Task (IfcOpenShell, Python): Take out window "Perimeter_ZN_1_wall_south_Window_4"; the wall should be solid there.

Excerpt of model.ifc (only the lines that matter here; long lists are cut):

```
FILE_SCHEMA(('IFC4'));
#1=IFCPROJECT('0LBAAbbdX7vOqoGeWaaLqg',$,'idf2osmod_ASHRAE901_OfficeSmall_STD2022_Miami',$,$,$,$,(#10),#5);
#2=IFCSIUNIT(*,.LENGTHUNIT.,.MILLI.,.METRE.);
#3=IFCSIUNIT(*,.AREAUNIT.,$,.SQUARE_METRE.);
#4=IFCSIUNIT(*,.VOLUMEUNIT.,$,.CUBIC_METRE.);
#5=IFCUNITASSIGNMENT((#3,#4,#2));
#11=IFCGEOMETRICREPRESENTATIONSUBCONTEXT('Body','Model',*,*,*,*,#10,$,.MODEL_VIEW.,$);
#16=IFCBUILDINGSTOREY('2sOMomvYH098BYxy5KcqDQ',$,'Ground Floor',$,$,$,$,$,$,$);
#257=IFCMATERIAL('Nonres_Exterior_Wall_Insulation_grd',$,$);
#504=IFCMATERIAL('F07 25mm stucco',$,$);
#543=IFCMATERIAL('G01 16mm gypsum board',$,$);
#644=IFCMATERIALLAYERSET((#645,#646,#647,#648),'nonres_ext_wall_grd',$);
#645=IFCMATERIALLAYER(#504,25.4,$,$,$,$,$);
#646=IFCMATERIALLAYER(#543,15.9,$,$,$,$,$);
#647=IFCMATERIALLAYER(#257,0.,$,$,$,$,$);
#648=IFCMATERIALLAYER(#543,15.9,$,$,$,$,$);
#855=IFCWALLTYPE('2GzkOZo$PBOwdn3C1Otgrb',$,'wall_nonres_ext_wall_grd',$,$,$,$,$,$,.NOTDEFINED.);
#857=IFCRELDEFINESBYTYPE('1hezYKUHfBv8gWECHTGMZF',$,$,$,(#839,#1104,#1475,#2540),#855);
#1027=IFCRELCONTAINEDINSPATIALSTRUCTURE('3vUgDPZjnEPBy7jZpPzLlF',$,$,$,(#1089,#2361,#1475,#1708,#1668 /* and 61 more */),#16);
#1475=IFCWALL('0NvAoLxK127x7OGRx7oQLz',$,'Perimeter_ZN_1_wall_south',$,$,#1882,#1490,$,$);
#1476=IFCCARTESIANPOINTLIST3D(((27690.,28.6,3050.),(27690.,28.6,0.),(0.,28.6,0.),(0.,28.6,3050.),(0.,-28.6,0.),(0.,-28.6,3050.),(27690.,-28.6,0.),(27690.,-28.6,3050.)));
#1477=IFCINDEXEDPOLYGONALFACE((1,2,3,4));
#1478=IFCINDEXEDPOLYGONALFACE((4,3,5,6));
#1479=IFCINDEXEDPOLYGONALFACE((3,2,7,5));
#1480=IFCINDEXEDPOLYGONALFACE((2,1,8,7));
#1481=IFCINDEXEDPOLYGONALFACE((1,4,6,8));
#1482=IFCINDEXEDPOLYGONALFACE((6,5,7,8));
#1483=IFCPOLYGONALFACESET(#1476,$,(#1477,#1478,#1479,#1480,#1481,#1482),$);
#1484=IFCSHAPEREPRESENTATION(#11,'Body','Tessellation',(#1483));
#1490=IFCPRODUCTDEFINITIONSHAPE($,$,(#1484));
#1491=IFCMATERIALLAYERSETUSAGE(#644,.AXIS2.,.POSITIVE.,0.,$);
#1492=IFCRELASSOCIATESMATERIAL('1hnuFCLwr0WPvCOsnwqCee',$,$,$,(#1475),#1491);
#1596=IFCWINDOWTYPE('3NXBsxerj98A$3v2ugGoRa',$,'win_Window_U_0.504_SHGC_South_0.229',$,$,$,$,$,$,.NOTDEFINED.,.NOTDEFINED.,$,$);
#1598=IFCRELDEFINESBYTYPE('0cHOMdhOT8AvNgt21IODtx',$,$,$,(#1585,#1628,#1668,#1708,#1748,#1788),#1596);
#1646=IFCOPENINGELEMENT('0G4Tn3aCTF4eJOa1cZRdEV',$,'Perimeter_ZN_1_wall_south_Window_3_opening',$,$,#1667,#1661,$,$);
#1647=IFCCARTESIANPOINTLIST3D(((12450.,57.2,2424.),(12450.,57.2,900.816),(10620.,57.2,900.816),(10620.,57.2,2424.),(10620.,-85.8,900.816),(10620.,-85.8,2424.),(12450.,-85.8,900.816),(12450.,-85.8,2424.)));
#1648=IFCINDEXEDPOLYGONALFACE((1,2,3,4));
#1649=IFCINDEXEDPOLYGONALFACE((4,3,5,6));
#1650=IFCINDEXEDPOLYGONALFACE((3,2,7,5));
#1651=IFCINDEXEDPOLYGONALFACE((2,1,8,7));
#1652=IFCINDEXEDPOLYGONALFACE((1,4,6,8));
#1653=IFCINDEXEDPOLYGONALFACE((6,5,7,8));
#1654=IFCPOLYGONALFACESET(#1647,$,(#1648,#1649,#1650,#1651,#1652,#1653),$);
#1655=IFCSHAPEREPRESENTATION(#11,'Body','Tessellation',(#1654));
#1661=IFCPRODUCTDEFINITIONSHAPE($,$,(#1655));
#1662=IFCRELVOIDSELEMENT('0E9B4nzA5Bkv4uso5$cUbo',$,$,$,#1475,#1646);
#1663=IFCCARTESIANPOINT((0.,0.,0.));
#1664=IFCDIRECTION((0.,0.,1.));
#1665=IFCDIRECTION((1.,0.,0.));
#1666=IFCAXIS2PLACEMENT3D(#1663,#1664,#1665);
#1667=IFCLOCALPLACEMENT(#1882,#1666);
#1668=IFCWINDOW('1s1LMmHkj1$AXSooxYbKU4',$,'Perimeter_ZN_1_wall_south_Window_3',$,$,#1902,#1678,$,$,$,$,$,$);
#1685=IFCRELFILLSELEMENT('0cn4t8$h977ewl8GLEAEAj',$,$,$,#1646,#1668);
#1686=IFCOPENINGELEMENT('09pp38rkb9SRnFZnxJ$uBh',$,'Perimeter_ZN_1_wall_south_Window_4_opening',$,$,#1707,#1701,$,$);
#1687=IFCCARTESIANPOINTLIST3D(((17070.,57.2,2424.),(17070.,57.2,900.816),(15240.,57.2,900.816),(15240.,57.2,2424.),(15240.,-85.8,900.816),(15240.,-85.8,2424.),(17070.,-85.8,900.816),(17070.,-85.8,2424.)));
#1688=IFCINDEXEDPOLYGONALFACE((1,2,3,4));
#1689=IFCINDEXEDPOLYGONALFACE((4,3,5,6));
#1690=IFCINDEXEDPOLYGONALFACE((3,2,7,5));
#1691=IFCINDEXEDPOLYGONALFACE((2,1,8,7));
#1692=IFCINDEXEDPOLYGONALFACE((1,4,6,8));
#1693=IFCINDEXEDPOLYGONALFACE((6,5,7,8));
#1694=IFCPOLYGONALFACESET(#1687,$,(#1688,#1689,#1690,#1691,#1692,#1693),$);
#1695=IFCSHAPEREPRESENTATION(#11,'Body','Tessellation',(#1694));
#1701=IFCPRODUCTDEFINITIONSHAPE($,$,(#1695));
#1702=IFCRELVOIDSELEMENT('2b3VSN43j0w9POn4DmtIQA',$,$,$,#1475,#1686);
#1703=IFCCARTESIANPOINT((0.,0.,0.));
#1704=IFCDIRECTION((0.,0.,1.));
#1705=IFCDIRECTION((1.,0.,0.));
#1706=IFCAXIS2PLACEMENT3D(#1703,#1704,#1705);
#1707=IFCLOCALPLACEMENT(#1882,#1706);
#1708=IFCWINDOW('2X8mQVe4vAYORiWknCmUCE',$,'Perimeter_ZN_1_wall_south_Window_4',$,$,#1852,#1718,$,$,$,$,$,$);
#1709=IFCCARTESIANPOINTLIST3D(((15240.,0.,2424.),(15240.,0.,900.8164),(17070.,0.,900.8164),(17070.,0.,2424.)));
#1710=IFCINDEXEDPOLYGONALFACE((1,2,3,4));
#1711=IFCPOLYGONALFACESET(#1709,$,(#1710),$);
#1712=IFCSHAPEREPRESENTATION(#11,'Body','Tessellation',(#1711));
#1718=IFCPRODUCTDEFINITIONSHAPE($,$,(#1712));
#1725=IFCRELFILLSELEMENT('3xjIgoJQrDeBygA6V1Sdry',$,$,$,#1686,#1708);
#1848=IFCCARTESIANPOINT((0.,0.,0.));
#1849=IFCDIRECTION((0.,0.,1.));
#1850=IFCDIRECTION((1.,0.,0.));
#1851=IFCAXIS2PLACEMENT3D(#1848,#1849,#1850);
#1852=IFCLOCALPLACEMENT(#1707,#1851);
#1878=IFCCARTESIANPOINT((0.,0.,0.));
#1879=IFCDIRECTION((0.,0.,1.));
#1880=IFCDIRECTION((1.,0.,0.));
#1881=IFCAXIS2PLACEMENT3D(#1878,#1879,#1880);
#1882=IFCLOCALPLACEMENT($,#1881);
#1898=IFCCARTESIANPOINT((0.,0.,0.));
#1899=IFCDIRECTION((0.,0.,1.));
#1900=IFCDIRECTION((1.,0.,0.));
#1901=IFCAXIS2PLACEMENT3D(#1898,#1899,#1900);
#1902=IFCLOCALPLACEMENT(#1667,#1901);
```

```python
import ifcopenshell
import ifcopenshell.api.feature
import ifcopenshell.api.root
import ifcopenshell.geom
import ifcopenshell.util.shape

model = ifcopenshell.open("model.ifc")
settings = ifcopenshell.geom.settings()


def volume(element):
    """Net volume in cubic metres, openings subtracted."""
    shape = ifcopenshell.geom.create_shape(settings, element)
    return ifcopenshell.util.shape.get_volume(shape.geometry)


window = model.by_guid("2X8mQVe4vAYORiWknCmUCE")
opening = window.FillsVoids[0].RelatingOpeningElement
wall = opening.VoidsElements[0].RelatingBuildingElement
before = volume(wall)

ifcopenshell.api.root.remove_product(model, product=window)
ifcopenshell.api.feature.remove_feature(model, feature=opening)

after = volume(wall)

print(f"wall volume {before:.3f} -> {after:.3f} m3")

model.write("model_v2.ifc")
```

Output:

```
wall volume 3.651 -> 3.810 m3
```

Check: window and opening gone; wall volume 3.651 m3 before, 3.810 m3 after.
